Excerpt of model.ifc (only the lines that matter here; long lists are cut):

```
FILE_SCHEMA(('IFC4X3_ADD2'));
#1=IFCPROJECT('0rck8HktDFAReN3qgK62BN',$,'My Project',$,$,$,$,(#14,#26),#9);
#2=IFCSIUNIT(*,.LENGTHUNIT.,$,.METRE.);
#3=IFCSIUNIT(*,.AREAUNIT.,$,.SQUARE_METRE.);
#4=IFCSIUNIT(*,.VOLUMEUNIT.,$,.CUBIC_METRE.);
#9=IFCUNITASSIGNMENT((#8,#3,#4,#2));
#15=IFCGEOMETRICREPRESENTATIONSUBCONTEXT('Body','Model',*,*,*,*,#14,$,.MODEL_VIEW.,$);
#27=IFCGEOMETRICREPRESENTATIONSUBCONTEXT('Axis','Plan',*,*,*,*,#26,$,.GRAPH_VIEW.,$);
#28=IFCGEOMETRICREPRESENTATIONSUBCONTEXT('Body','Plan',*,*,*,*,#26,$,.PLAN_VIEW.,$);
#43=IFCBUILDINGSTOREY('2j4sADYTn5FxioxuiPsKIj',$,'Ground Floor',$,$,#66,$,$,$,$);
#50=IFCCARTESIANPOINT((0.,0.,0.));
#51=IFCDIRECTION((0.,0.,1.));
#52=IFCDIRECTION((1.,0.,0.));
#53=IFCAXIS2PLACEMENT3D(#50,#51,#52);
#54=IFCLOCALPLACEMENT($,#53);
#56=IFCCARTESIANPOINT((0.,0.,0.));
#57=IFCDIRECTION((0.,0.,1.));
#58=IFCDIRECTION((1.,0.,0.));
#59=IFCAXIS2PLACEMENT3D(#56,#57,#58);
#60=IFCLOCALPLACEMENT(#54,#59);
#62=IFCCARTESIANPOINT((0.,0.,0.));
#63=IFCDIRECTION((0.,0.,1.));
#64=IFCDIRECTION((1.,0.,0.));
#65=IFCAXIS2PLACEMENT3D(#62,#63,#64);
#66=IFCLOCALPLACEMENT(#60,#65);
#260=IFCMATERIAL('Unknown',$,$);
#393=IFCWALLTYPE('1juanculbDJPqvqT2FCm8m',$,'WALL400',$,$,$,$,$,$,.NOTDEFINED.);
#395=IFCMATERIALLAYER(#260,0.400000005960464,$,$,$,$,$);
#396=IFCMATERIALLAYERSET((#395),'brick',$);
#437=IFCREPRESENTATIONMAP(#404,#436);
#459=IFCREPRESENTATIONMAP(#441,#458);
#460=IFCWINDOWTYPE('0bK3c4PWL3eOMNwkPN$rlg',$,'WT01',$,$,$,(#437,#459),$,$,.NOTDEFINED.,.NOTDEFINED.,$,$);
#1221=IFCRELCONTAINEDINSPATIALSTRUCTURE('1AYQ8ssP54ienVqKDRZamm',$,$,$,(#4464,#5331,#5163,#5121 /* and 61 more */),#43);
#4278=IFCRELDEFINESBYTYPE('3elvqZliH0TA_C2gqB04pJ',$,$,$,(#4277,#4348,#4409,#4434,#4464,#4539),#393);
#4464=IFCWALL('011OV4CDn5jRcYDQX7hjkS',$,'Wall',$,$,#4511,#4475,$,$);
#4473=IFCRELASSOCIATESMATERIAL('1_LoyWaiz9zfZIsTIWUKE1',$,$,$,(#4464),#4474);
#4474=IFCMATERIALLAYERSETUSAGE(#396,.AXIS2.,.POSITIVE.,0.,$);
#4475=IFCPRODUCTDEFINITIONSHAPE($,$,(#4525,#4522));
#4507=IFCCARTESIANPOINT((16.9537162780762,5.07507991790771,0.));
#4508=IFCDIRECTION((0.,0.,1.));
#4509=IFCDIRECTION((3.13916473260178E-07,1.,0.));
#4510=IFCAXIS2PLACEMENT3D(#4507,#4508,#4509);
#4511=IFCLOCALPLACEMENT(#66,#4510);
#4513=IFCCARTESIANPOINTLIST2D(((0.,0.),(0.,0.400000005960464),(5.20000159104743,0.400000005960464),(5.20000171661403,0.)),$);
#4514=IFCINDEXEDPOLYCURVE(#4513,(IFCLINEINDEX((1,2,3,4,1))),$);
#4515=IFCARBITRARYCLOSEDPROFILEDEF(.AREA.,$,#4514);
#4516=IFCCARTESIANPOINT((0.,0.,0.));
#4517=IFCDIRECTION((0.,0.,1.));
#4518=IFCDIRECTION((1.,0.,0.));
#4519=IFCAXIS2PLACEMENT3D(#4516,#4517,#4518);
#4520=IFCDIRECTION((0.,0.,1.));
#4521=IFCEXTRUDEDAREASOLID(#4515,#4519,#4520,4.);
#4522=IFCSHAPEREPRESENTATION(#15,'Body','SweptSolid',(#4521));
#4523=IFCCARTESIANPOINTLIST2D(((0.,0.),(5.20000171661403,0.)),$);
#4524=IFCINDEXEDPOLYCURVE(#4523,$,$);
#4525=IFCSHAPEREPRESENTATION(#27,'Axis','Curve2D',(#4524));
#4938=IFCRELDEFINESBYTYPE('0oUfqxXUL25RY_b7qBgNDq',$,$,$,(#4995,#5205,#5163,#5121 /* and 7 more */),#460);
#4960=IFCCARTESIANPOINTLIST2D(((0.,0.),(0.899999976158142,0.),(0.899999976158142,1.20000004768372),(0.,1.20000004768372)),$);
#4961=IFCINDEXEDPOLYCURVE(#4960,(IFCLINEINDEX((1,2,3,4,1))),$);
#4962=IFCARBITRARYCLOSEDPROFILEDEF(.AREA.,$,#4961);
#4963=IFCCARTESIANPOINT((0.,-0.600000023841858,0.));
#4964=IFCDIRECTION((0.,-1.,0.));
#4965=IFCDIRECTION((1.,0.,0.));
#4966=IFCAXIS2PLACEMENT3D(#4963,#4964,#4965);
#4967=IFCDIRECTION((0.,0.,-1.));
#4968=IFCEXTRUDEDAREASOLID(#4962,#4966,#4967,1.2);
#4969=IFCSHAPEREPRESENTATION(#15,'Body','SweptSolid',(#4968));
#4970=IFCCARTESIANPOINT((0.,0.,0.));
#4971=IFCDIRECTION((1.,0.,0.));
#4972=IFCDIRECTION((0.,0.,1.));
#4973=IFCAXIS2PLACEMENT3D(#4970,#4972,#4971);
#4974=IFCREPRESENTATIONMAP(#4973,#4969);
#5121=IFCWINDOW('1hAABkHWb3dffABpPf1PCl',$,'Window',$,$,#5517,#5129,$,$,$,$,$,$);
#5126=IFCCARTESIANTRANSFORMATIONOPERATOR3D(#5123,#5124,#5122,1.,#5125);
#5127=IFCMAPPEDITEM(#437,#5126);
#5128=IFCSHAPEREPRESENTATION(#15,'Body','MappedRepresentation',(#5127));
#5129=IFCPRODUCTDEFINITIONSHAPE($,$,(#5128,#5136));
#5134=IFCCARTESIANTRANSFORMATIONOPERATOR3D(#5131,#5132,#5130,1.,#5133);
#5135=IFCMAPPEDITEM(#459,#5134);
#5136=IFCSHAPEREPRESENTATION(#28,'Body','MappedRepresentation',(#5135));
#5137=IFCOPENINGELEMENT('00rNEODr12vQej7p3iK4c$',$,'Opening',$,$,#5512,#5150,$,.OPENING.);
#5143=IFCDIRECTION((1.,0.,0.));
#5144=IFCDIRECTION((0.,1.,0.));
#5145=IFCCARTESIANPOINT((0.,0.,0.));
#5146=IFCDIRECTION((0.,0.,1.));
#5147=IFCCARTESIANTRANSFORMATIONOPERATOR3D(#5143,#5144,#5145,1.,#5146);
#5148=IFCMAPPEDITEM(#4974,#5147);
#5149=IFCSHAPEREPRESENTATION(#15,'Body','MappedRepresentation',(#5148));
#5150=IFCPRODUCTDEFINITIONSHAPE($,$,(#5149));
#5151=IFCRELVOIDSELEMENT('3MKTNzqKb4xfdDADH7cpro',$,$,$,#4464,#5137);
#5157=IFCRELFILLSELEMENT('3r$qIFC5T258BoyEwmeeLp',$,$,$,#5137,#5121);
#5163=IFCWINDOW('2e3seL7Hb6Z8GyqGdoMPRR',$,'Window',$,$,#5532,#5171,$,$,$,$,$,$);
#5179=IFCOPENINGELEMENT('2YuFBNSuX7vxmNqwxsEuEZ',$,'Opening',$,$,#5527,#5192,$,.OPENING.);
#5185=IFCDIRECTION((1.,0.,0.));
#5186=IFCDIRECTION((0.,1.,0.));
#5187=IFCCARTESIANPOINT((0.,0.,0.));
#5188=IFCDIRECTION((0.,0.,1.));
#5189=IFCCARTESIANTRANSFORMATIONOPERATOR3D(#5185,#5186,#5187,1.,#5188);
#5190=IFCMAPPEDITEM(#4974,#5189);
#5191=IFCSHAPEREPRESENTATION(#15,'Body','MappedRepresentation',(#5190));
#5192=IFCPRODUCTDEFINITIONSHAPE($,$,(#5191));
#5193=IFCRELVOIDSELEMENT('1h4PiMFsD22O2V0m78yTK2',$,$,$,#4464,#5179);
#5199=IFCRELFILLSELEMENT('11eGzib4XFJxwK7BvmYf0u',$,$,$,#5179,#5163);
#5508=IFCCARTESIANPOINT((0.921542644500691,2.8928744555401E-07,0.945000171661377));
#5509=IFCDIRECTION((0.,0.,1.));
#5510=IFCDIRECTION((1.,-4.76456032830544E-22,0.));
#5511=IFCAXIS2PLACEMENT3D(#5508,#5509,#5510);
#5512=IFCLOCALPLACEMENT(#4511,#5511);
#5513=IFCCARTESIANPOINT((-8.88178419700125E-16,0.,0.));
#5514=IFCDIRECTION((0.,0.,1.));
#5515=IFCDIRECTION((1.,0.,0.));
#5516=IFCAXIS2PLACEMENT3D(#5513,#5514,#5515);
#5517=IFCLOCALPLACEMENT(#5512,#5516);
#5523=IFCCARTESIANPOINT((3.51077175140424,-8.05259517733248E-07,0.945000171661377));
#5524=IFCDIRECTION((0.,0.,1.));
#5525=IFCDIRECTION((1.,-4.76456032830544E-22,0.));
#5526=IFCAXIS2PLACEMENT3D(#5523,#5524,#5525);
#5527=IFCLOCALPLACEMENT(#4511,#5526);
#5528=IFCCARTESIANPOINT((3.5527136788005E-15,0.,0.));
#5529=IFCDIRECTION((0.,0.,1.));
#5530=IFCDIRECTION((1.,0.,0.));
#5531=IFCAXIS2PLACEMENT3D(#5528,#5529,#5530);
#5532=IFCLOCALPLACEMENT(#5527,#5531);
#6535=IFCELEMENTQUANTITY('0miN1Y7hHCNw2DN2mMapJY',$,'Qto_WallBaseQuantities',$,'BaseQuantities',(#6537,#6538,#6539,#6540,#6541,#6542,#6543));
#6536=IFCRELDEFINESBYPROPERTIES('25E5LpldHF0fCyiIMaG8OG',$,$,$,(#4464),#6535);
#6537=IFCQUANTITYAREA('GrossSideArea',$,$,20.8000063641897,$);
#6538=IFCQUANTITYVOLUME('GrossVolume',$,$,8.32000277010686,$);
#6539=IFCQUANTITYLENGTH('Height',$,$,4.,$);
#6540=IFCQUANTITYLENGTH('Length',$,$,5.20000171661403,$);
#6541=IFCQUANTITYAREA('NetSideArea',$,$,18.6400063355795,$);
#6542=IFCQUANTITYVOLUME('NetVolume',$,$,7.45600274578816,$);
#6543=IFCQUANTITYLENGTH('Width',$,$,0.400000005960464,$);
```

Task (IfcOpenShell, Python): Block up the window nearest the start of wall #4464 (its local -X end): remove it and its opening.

```python
import ifcopenshell
import ifcopenshell.api.feature
import ifcopenshell.api.pset
import ifcopenshell.api.root
import ifcopenshell.geom
import ifcopenshell.util.element
import ifcopenshell.util.shape
import ifcopenshell.util.unit

model = ifcopenshell.open("model.ifc")
area_scale = ifcopenshell.util.unit.calculate_unit_scale(model, "AREAUNIT")
volume_scale = ifcopenshell.util.unit.calculate_unit_scale(model, "VOLUMEUNIT")
settings = ifcopenshell.geom.settings()


def volume(element):
    """Net volume in cubic metres, openings subtracted."""
    shape = ifcopenshell.geom.create_shape(settings, element)
    return ifcopenshell.util.shape.get_volume(shape.geometry)


window = model.by_guid("1hAABkHWb3dffABpPf1PCl")
opening = window.FillsVoids[0].RelatingOpeningElement
wall = opening.VoidsElements[0].RelatingBuildingElement
before = volume(wall)

ifcopenshell.api.root.remove_product(model, product=window)
ifcopenshell.api.feature.remove_feature(model, feature=opening)

after = volume(wall)
thickness = 0.4  # wall thickness in metres

# Update the wall's stored quantities.
qto = model.by_id(ifcopenshell.util.element.get_pset(wall, "Qto_WallBaseQuantities", should_inherit=False)["id"])
ifcopenshell.api.pset.edit_qto(model, qto=qto, properties={
    "NetSideArea": after / thickness / area_scale,
    "NetVolume": after / volume_scale,
})

print(f"wall volume {before:.3f} -> {after:.3f} m3")

model.write("model_v2.ifc")
```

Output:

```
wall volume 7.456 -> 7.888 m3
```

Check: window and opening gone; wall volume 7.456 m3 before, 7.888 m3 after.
